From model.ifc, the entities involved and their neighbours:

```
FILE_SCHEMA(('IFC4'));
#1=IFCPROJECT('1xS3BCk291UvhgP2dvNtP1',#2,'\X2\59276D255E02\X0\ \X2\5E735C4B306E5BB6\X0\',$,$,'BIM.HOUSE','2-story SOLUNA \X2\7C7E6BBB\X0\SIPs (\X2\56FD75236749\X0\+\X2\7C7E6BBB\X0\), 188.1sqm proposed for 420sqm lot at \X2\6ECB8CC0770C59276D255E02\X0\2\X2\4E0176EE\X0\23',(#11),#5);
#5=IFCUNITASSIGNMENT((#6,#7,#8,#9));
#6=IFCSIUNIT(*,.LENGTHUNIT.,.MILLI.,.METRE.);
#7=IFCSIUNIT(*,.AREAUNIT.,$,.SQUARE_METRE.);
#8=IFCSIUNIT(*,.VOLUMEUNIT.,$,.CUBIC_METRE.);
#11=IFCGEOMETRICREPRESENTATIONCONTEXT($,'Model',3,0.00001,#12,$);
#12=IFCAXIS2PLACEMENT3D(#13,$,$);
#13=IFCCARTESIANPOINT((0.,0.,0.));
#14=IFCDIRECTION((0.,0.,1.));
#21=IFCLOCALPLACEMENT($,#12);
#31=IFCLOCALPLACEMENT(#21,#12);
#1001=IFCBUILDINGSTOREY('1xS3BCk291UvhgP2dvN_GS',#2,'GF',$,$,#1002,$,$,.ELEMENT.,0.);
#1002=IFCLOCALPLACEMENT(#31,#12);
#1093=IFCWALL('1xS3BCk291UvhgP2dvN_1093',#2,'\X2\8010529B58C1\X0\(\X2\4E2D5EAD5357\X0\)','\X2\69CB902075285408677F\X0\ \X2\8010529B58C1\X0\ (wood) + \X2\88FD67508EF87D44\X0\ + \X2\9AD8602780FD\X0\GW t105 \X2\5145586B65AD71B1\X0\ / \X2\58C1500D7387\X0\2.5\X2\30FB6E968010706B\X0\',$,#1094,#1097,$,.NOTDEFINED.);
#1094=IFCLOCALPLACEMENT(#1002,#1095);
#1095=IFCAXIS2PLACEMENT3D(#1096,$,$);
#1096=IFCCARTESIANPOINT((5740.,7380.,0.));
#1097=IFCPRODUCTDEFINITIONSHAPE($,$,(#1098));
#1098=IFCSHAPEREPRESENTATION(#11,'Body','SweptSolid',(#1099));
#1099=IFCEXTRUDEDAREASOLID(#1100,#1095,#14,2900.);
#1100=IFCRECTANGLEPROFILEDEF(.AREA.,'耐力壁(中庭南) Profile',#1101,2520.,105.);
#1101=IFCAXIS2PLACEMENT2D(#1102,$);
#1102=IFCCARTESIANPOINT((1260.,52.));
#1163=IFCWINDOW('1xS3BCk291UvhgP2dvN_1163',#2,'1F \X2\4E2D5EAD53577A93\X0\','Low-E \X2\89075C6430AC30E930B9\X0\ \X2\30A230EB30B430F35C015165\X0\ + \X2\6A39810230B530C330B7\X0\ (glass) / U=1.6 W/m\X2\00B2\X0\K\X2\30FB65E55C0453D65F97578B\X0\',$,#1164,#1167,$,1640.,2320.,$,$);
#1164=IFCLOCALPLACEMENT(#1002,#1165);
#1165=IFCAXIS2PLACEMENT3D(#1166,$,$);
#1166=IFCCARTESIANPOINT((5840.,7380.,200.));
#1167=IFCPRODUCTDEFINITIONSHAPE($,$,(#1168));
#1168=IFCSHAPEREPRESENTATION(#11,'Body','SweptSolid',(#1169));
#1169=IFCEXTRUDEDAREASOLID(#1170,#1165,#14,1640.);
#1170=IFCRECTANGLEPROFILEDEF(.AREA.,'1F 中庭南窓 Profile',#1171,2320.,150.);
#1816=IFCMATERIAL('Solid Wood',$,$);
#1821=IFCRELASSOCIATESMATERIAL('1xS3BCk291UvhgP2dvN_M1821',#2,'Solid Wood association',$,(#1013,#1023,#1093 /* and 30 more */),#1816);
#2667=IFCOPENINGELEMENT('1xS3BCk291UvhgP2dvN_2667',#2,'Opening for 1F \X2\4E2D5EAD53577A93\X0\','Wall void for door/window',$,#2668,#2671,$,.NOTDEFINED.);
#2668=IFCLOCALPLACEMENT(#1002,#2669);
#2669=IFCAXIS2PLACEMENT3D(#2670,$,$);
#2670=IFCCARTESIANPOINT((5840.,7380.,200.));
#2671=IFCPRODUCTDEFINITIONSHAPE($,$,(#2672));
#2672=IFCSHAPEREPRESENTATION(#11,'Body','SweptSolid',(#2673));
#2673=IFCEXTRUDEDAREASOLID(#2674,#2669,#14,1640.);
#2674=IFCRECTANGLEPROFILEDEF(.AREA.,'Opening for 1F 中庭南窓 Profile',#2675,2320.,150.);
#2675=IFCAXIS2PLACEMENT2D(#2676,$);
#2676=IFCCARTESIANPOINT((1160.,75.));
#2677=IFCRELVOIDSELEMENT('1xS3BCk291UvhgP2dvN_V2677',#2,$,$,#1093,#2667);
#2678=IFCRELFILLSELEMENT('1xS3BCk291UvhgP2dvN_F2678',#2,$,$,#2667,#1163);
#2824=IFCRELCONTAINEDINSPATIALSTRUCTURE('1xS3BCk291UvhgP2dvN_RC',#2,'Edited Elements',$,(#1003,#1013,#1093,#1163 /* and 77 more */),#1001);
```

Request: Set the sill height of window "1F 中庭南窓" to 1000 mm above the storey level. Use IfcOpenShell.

```python
import numpy as np
import ifcopenshell
import ifcopenshell.api.geometry
import ifcopenshell.geom
import ifcopenshell.util.element
import ifcopenshell.util.placement
import ifcopenshell.util.shape
import ifcopenshell.util.unit

model = ifcopenshell.open("model.ifc")
unit_scale = ifcopenshell.util.unit.calculate_unit_scale(model)

window = model.by_guid("1xS3BCk291UvhgP2dvN_1163")
opening = window.FillsVoids[0].RelatingOpeningElement
storey = ifcopenshell.util.element.get_container(window, ifc_class="IfcBuildingStorey")
level = ifcopenshell.util.placement.get_local_placement(storey.ObjectPlacement)[2, 3]

# The opening's origin need not be at the sill, so measure its lowest point.
shape = ifcopenshell.geom.create_shape(ifcopenshell.geom.settings(), opening)
bottom = ifcopenshell.util.shape.get_shape_bottom_elevation(shape, shape.geometry) / unit_scale
dz = level + 1 / unit_scale - bottom

shift = np.array([0.0, 0.0, dz])
# The window is not placed relative to its opening, so move both.
for product in (opening, window):
    matrix = ifcopenshell.util.placement.get_local_placement(product.ObjectPlacement)
    matrix[:3, 3] += shift
    ifcopenshell.api.geometry.edit_object_placement(model, product=product, matrix=matrix, is_si=False)

print(f"moved by {dz * unit_scale:+.3f} m")

model.write("model_v2.ifc")
```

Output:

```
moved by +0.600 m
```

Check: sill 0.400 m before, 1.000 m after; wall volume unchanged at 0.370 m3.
